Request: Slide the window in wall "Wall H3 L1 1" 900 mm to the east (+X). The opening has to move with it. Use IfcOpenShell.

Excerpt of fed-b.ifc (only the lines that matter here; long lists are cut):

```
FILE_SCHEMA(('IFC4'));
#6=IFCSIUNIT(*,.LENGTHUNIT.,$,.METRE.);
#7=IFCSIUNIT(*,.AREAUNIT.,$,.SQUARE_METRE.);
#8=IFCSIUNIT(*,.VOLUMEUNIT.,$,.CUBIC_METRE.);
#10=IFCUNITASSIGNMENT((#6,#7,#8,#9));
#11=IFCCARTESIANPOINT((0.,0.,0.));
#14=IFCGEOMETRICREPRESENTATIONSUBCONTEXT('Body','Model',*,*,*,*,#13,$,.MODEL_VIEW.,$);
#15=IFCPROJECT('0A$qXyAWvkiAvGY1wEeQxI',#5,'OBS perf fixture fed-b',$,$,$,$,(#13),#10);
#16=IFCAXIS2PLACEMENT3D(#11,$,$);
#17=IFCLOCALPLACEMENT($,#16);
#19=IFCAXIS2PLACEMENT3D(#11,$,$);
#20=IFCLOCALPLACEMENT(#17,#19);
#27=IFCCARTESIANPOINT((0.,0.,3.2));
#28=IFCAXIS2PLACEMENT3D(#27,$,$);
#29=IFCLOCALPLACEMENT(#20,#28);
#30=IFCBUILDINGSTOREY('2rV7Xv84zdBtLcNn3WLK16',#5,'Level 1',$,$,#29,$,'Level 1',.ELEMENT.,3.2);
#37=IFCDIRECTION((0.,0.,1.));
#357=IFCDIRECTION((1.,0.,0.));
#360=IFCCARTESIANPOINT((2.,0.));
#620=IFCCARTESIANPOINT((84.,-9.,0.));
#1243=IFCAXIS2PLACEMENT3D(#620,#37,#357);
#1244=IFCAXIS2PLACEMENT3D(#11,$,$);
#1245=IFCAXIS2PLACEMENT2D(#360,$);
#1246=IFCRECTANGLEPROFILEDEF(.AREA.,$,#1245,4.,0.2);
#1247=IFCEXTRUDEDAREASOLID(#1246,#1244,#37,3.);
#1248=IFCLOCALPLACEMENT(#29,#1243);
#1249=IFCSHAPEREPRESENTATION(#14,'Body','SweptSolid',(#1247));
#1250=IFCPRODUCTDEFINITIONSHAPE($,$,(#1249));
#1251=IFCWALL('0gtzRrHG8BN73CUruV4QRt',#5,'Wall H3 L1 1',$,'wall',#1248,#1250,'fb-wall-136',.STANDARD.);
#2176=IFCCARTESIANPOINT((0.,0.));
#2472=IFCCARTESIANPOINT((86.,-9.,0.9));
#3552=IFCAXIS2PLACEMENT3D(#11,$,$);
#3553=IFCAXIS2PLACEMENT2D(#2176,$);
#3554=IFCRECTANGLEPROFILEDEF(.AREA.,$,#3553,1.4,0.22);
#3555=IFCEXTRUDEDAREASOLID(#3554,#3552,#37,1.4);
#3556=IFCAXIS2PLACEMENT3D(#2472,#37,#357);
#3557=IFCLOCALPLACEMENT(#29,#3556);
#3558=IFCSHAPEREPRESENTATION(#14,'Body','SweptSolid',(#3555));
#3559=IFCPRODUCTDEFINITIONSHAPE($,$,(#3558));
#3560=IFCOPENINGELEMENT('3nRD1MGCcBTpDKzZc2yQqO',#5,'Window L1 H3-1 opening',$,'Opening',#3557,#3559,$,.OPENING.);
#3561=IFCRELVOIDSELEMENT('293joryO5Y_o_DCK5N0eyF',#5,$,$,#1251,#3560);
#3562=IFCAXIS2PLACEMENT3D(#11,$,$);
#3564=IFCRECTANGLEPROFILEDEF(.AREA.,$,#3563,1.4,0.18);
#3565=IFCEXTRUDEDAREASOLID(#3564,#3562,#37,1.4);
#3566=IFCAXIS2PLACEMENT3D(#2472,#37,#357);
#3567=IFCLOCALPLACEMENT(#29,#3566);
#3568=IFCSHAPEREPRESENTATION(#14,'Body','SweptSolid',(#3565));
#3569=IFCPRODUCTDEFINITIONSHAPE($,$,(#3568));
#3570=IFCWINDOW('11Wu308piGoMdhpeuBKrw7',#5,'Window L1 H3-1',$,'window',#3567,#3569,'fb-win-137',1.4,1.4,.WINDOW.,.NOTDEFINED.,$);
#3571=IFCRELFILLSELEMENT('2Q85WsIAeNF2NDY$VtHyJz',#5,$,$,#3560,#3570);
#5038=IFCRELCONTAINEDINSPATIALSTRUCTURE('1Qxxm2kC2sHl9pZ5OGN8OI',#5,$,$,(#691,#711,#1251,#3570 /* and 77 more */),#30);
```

```python
import ifcopenshell
import ifcopenshell.api.geometry
import ifcopenshell.util.placement

model = ifcopenshell.open("fed-b.ifc")

window = model.by_id(3570)
opening = window.FillsVoids[0].RelatingOpeningElement
wall = opening.VoidsElements[0].RelatingBuildingElement

wall_matrix = ifcopenshell.util.placement.get_local_placement(wall.ObjectPlacement)
shift = wall_matrix[:3, 0] * 0.9
before = ifcopenshell.util.placement.get_local_placement(window.ObjectPlacement)[:3, 3].copy()

# The window is not placed relative to its opening, so move both.
for product in (opening, window):
    matrix = ifcopenshell.util.placement.get_local_placement(product.ObjectPlacement)
    matrix[:3, 3] += shift
    ifcopenshell.api.geometry.edit_object_placement(model, product=product, matrix=matrix, is_si=False)

after = ifcopenshell.util.placement.get_local_placement(window.ObjectPlacement)[:3, 3]
print("window moved by", (after - before).round(3) + 0.0)

model.write("fed-b_rev.ifc")
```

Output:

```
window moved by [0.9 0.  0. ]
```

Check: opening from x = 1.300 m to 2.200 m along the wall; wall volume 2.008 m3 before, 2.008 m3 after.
